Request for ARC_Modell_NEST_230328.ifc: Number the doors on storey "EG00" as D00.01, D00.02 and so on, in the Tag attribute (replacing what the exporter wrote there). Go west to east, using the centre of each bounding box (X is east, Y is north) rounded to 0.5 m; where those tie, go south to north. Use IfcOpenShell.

First a look at what the model holds.

```python
import ifcopenshell
import ifcopenshell.util.element
import ifcopenshell.util.placement

model = ifcopenshell.open("ARC_Modell_NEST_230328.ifc")
print(model.schema)
storey = next(s for s in model.by_type("IfcBuildingStorey") if s.Name == "EG00")
doors = [e for e in ifcopenshell.util.element.get_decomposition(storey) if e.is_a("IfcDoor")]
for e in sorted(doors, key=lambda e: e.id()):
    origin = ifcopenshell.util.placement.get_local_placement(e.ObjectPlacement)[:3, 3]
    print(e.id(), e.Tag, e.Name, origin.round(2) + 0.0, sep=" | ")
```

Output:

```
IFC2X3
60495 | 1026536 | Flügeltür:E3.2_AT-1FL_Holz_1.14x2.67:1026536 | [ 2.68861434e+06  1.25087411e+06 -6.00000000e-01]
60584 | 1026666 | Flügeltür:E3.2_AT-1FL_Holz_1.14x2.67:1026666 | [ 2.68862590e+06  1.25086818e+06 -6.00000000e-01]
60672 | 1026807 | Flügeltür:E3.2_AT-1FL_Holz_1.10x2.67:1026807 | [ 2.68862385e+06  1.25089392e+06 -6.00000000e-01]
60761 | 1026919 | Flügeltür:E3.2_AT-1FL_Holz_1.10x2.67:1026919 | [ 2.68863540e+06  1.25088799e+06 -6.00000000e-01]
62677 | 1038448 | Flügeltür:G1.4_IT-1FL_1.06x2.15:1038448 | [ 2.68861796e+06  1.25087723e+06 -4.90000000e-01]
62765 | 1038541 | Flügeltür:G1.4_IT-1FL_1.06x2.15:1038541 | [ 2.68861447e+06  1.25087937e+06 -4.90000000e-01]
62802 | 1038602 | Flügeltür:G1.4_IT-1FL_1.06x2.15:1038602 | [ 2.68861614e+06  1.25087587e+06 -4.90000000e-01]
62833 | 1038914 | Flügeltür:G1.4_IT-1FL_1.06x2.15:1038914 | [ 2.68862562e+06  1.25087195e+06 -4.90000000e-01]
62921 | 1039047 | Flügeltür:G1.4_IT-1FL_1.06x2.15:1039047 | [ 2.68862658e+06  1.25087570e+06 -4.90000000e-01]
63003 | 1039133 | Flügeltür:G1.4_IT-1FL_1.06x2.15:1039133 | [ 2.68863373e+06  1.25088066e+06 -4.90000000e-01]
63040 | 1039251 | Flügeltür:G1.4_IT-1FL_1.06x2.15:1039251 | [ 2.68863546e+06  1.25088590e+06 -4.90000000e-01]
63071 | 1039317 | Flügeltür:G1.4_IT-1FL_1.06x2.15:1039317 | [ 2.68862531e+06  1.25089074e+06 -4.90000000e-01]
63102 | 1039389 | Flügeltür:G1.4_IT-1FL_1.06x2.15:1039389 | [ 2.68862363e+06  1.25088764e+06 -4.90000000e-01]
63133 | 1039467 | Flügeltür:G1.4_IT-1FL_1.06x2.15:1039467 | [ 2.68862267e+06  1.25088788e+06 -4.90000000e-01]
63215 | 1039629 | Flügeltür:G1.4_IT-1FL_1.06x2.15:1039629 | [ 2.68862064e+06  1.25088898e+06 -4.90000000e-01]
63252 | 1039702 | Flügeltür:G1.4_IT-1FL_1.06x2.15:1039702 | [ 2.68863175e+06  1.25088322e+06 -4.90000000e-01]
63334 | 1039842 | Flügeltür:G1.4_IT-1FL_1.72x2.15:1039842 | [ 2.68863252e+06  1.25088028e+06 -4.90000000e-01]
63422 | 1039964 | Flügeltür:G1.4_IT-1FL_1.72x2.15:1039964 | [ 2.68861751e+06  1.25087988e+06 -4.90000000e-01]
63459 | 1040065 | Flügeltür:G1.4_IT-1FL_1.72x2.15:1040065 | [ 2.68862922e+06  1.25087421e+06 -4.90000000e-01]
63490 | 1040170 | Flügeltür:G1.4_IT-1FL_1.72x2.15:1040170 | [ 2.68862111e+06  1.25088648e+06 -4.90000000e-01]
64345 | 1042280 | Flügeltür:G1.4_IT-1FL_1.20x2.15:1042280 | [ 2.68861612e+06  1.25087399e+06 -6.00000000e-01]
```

```python
import ifcopenshell
import ifcopenshell.geom
import ifcopenshell.util.element
import ifcopenshell.util.shape

model = ifcopenshell.open("ARC_Modell_NEST_230328.ifc")
settings = ifcopenshell.geom.settings()
settings.set("use-world-coords", True)


def centre(element):
    shape = ifcopenshell.geom.create_shape(settings, element)
    return ifcopenshell.util.shape.get_bbox_centroid(shape.geometry)


storey = next(s for s in model.by_type("IfcBuildingStorey") if s.Name == "EG00")
doors = [e for e in ifcopenshell.util.element.get_decomposition(storey) if e.is_a("IfcDoor")]

# Insertion points can sit at a corner or the storey origin, so sort by the geometry (in metres).
centres = {e: centre(e) for e in doors}
doors.sort(key=lambda e: (round(centres[e][0] / 0.5), centres[e][1]))

for i, e in enumerate(doors, start=1):
    number = f"D00.{i:02d}"
    e.Tag = number
    print(e.id(), number)

model.write("ARC_Modell_NEST_230328_edited.ifc")
```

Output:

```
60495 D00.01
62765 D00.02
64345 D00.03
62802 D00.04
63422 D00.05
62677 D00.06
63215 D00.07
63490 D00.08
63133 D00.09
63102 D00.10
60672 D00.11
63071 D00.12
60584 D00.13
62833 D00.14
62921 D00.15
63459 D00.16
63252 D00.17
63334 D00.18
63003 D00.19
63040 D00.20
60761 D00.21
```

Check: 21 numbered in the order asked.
